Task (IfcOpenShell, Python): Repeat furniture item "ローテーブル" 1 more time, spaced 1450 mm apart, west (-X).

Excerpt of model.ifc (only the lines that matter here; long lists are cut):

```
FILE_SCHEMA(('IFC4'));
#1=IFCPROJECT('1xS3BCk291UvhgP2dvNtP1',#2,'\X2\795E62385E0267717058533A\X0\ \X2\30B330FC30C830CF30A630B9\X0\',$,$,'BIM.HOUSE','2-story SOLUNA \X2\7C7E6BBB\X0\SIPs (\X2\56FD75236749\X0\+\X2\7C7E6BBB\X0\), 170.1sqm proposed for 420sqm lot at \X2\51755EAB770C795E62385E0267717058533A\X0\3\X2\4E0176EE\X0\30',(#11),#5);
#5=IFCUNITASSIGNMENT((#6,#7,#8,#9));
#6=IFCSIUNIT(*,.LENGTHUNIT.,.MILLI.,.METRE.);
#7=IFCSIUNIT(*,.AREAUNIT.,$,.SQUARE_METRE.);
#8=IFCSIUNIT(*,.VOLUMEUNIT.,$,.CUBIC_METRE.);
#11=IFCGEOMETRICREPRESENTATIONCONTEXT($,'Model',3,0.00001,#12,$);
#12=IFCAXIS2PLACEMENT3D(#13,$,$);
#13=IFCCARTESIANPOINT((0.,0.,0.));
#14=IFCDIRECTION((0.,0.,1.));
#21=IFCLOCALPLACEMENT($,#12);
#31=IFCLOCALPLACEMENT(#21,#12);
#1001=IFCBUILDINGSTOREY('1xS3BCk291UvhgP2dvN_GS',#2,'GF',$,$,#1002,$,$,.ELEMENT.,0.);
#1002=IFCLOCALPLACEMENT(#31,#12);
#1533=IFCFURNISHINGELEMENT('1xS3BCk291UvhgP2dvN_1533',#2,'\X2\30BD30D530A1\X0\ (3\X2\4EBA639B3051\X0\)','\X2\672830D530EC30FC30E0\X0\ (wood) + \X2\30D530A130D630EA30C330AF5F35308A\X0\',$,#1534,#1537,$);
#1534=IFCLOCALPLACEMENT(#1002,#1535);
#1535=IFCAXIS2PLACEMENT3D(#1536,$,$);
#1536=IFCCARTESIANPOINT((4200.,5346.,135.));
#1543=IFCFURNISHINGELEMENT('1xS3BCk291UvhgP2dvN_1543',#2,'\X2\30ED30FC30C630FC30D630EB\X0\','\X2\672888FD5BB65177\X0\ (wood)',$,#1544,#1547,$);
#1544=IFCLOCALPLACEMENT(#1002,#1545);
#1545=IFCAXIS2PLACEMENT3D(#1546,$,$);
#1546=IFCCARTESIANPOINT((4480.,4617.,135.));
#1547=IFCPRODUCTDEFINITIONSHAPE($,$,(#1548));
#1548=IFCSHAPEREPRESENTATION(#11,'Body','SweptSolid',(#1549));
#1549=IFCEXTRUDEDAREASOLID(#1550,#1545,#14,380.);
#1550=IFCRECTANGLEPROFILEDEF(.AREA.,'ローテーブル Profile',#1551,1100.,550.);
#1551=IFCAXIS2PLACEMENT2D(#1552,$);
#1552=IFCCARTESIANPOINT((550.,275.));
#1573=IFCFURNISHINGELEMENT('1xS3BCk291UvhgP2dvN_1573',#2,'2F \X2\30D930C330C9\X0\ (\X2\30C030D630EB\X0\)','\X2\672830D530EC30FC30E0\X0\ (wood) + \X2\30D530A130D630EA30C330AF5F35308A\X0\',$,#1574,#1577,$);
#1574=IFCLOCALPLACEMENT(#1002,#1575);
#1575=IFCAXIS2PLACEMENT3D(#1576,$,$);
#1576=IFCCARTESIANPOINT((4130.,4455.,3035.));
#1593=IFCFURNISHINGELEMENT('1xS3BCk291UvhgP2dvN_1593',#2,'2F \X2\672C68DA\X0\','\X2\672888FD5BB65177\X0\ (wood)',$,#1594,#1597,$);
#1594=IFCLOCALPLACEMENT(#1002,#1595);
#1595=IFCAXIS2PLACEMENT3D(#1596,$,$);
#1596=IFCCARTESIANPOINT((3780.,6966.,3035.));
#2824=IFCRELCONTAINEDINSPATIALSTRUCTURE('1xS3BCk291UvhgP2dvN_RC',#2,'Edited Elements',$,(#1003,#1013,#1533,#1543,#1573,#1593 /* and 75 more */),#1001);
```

```python
import numpy as np
import ifcopenshell
import ifcopenshell.api.geometry
import ifcopenshell.api.root
import ifcopenshell.util.element
import ifcopenshell.util.placement
import ifcopenshell.util.unit

model = ifcopenshell.open("model.ifc")
unit_scale = ifcopenshell.util.unit.calculate_unit_scale(model)


def reuse_history(source, copy):
    """copy_class also copies each property set's owner history, people and application; keep the originals."""
    for rel in copy.IsDefinedBy:
        if rel.is_a("IfcRelDefinesByProperties") and (history := rel.RelatingPropertyDefinition.OwnerHistory):
            rel.RelatingPropertyDefinition.OwnerHistory = source.OwnerHistory
            ifcopenshell.util.element.remove_deep2(model, history)


source = model.by_guid("1xS3BCk291UvhgP2dvN_1543")
base = ifcopenshell.util.placement.get_local_placement(source.ObjectPlacement)
step = np.array([-1.0, 0.0, 0.0]) * 1.45 / unit_scale

for i in range(1, 2):
    copy = ifcopenshell.api.root.copy_class(model, product=source)
    copy.Representation = ifcopenshell.util.element.copy_deep(
        model, source.Representation, exclude=["IfcGeometricRepresentationContext", "IfcRepresentationMap"]
    )
    reuse_history(source, copy)
    matrix = base.copy()
    matrix[:3, 3] += i * step
    print("added at", matrix[:3, 3].round(3) + 0.0)
    ifcopenshell.api.geometry.edit_object_placement(model, product=copy, matrix=matrix, is_si=False)

model.write("model_rev.ifc")
```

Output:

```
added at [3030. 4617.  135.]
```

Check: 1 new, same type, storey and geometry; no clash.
